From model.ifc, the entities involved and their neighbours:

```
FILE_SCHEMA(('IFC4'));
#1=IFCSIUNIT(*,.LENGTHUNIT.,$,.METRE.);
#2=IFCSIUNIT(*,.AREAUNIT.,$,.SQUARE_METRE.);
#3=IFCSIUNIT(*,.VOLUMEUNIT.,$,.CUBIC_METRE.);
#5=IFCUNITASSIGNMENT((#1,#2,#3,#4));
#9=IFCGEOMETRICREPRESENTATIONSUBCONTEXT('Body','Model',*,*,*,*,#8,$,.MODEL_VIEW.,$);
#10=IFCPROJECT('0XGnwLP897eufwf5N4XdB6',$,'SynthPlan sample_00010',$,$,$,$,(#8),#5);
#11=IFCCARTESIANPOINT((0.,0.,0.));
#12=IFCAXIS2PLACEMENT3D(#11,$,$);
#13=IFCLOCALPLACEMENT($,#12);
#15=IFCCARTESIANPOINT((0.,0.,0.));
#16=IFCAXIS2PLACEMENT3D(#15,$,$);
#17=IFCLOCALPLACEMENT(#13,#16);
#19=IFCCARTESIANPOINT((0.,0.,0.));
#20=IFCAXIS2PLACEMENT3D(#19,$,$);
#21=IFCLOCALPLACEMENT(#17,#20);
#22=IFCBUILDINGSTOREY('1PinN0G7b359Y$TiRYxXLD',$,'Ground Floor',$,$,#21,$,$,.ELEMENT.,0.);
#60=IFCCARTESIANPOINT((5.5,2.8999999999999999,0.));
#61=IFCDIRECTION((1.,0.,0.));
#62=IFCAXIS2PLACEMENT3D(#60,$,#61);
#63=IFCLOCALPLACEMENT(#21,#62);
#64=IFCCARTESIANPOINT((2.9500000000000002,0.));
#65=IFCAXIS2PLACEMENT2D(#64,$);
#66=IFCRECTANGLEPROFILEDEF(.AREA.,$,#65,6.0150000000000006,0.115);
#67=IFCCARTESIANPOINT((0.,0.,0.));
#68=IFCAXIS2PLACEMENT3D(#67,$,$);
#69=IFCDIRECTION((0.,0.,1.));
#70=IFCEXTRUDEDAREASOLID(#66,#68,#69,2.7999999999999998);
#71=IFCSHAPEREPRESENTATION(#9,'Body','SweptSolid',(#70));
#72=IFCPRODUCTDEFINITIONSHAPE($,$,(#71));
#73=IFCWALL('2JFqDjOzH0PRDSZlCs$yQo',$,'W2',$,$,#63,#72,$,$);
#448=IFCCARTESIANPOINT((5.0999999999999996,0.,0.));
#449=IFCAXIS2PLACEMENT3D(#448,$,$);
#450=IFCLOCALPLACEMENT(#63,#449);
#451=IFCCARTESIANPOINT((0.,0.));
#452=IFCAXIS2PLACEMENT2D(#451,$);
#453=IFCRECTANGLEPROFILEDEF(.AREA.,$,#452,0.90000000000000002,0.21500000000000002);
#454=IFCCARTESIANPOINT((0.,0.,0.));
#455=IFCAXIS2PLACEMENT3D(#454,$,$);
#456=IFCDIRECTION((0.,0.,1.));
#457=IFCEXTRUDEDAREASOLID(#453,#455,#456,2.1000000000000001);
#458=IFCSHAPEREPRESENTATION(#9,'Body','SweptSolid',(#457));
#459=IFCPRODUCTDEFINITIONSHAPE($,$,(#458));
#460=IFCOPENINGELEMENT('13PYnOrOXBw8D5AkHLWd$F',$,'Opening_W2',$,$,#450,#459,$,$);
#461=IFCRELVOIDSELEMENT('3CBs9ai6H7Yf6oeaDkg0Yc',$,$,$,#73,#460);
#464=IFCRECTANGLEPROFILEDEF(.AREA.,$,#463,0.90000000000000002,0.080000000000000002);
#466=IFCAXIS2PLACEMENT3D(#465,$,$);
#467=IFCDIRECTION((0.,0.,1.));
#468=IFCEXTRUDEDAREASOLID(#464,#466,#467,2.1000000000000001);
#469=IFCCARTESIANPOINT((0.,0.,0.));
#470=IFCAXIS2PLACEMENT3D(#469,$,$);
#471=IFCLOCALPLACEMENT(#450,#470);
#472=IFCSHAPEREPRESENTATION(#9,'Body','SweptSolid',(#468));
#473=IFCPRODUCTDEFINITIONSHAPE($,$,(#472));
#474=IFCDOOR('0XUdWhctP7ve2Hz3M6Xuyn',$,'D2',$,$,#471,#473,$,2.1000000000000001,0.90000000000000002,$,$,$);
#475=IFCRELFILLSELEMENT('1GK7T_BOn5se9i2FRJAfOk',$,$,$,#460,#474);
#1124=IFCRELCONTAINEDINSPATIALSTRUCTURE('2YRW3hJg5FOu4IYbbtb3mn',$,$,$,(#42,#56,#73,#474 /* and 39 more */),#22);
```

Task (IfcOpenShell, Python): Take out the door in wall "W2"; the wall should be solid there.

```python
import ifcopenshell
import ifcopenshell.api.feature
import ifcopenshell.api.root
import ifcopenshell.geom
import ifcopenshell.util.shape

model = ifcopenshell.open("model.ifc")
settings = ifcopenshell.geom.settings()


def volume(element):
    """Net volume in cubic metres, openings subtracted."""
    shape = ifcopenshell.geom.create_shape(settings, element)
    return ifcopenshell.util.shape.get_volume(shape.geometry)


door = model.by_guid("0XUdWhctP7ve2Hz3M6Xuyn")
opening = door.FillsVoids[0].RelatingOpeningElement
wall = opening.VoidsElements[0].RelatingBuildingElement
before = volume(wall)

ifcopenshell.api.root.remove_product(model, product=door)
ifcopenshell.api.feature.remove_feature(model, feature=opening)

after = volume(wall)

print(f"wall volume {before:.3f} -> {after:.3f} m3")

model.write("model_v2.ifc")
```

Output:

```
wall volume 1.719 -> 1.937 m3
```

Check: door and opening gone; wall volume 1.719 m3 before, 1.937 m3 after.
